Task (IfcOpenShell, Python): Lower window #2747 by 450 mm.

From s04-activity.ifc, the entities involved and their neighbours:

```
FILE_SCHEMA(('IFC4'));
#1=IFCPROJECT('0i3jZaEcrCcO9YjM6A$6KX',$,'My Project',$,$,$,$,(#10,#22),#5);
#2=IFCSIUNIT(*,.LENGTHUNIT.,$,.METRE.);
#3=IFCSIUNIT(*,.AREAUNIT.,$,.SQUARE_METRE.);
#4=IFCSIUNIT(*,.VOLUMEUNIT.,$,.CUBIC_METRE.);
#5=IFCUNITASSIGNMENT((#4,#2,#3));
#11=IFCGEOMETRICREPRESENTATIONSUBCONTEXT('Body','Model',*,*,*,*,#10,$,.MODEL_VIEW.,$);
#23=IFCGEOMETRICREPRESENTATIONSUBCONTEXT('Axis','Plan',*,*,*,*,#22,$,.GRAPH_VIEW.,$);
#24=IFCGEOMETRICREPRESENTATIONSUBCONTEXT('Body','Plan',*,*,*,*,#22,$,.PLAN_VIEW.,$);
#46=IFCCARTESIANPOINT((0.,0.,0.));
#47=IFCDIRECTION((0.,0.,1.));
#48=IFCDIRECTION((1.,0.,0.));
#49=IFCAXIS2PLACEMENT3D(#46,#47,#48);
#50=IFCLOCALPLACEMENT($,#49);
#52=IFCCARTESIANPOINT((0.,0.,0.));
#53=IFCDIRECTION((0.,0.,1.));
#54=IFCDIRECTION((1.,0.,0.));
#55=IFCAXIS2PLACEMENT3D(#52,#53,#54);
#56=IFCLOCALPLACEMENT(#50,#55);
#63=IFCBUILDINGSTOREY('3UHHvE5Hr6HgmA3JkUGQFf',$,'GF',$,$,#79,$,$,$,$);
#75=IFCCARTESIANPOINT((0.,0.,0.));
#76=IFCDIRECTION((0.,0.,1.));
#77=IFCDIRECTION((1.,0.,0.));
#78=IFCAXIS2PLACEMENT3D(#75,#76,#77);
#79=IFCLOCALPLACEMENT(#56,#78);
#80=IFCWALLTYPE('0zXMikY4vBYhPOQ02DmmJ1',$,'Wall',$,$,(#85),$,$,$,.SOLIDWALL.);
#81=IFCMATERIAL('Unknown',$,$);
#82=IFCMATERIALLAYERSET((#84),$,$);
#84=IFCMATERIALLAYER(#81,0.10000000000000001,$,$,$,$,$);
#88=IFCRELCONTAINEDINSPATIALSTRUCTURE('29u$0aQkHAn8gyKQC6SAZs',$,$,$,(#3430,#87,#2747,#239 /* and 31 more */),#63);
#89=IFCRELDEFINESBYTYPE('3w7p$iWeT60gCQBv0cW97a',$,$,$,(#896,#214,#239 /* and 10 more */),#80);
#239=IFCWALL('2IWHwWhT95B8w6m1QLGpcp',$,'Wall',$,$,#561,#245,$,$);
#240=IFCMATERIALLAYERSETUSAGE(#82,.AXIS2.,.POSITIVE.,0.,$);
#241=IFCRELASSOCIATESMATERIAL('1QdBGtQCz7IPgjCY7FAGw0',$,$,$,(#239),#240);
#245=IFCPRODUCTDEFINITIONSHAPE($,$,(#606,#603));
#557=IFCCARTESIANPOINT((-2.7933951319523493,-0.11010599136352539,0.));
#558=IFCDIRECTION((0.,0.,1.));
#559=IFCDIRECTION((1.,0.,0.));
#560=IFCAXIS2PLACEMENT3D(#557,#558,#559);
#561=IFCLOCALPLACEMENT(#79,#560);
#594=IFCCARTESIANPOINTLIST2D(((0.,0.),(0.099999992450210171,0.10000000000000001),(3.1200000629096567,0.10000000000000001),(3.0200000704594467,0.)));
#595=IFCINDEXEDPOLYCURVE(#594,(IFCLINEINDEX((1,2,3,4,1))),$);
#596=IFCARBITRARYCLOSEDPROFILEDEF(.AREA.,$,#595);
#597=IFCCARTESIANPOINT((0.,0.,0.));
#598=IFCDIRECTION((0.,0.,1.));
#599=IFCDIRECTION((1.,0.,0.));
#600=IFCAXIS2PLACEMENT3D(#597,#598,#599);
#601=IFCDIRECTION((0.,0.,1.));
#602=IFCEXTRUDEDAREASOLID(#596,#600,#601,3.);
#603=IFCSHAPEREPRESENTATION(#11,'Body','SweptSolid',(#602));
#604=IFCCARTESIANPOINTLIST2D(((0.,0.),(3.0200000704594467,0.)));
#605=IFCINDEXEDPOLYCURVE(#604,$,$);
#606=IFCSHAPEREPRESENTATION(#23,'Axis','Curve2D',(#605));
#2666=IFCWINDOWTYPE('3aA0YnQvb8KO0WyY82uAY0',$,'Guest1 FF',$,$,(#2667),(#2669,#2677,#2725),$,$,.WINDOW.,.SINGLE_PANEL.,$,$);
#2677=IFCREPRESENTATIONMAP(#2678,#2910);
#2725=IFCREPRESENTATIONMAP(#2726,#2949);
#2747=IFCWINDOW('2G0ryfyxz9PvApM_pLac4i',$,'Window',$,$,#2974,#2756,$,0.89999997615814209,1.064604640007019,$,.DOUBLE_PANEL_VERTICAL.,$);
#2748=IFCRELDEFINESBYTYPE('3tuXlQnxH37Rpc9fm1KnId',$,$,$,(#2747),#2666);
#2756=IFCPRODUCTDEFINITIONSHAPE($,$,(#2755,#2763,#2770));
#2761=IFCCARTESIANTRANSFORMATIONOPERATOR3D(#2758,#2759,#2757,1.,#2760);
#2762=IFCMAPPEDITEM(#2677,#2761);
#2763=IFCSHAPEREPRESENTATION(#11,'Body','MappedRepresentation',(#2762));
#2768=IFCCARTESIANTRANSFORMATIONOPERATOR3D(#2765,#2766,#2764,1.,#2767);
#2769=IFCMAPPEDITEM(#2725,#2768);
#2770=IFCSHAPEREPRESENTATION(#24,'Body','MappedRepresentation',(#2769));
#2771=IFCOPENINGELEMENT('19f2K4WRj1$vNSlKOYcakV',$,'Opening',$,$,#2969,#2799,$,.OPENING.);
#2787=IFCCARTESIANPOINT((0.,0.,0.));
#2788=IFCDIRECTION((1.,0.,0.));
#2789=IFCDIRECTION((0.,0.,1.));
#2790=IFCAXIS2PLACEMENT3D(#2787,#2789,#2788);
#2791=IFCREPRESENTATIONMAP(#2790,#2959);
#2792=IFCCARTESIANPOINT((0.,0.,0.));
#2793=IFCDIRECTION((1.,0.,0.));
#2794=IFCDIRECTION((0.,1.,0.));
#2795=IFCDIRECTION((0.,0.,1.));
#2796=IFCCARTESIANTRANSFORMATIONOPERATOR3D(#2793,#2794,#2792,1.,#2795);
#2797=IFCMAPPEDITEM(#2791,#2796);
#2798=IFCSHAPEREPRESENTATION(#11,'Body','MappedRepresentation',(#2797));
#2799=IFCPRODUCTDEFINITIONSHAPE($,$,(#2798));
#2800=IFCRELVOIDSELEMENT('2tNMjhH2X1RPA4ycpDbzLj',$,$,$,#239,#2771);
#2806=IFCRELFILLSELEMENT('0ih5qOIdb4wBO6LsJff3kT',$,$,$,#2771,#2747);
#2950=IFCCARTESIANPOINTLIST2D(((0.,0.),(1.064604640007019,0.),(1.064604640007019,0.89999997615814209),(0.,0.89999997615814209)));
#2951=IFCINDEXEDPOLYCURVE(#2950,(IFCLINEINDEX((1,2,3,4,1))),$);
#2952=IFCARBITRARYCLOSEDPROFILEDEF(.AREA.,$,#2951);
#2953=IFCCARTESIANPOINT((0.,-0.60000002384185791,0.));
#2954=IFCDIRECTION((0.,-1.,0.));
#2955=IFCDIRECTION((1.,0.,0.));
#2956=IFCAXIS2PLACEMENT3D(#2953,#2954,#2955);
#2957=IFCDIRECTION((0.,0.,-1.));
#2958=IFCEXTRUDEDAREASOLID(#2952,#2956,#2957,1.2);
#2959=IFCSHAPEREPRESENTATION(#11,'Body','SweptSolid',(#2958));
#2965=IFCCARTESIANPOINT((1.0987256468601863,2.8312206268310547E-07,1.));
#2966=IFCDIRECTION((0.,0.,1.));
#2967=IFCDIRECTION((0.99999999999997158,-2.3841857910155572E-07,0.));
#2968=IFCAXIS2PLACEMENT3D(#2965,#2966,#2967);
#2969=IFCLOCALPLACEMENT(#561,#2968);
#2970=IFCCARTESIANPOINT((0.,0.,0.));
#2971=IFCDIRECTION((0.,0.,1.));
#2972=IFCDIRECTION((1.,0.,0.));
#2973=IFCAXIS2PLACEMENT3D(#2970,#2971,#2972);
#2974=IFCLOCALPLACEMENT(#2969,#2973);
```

```python
import numpy as np
import ifcopenshell
import ifcopenshell.api.geometry
import ifcopenshell.util.placement
import ifcopenshell.util.unit

model = ifcopenshell.open("s04-activity.ifc")
unit_scale = ifcopenshell.util.unit.calculate_unit_scale(model)

window = model.by_id(2747)
opening = window.FillsVoids[0].RelatingOpeningElement
dz = -0.45

shift = np.array([0.0, 0.0, dz])
# The window is placed relative to its opening, so it follows when the opening moves.
matrix = ifcopenshell.util.placement.get_local_placement(opening.ObjectPlacement)
matrix[:3, 3] += shift
ifcopenshell.api.geometry.edit_object_placement(
    model, product=opening, matrix=matrix, is_si=False, should_transform_children=True
)

print(f"moved by {dz * unit_scale:+.3f} m")

model.write("s04-activity_edited.ifc")
```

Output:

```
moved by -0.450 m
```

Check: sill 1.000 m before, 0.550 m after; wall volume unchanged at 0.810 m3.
